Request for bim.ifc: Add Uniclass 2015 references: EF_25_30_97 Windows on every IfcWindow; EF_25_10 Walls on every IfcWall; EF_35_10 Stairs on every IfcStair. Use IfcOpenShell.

First a look at what the model holds.

```python
import ifcopenshell

model = ifcopenshell.open("bim.ifc")
print(model.schema)
print("classifications:", [c.Name for c in model.by_type("IfcClassification")])
for ifc_class in ("IfcDoor", "IfcRoof", "IfcStair", "IfcWall", "IfcWindow"):
    print(ifc_class, len(model.by_type(ifc_class)))
```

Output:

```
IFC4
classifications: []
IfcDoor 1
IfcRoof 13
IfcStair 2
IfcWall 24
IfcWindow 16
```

```python
import ifcopenshell
import ifcopenshell.api.classification

model = ifcopenshell.open("bim.ifc")

system = ifcopenshell.api.classification.add_classification(model, classification="Uniclass 2015")

codes = {
    "IfcWindow": ("EF_25_30_97", "Windows"),
    "IfcWall": ("EF_25_10", "Walls"),
    "IfcStair": ("EF_35_10", "Stairs"),
}
for ifc_class, (code, name) in codes.items():
    products = model.by_type(ifc_class)
    ifcopenshell.api.classification.add_reference(
        model, products=products, classification=system, identification=code, name=name
    )
    print(code, len(products))

model.write("bim_rev.ifc")
```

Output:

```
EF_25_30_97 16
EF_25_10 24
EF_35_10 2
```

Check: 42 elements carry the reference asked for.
